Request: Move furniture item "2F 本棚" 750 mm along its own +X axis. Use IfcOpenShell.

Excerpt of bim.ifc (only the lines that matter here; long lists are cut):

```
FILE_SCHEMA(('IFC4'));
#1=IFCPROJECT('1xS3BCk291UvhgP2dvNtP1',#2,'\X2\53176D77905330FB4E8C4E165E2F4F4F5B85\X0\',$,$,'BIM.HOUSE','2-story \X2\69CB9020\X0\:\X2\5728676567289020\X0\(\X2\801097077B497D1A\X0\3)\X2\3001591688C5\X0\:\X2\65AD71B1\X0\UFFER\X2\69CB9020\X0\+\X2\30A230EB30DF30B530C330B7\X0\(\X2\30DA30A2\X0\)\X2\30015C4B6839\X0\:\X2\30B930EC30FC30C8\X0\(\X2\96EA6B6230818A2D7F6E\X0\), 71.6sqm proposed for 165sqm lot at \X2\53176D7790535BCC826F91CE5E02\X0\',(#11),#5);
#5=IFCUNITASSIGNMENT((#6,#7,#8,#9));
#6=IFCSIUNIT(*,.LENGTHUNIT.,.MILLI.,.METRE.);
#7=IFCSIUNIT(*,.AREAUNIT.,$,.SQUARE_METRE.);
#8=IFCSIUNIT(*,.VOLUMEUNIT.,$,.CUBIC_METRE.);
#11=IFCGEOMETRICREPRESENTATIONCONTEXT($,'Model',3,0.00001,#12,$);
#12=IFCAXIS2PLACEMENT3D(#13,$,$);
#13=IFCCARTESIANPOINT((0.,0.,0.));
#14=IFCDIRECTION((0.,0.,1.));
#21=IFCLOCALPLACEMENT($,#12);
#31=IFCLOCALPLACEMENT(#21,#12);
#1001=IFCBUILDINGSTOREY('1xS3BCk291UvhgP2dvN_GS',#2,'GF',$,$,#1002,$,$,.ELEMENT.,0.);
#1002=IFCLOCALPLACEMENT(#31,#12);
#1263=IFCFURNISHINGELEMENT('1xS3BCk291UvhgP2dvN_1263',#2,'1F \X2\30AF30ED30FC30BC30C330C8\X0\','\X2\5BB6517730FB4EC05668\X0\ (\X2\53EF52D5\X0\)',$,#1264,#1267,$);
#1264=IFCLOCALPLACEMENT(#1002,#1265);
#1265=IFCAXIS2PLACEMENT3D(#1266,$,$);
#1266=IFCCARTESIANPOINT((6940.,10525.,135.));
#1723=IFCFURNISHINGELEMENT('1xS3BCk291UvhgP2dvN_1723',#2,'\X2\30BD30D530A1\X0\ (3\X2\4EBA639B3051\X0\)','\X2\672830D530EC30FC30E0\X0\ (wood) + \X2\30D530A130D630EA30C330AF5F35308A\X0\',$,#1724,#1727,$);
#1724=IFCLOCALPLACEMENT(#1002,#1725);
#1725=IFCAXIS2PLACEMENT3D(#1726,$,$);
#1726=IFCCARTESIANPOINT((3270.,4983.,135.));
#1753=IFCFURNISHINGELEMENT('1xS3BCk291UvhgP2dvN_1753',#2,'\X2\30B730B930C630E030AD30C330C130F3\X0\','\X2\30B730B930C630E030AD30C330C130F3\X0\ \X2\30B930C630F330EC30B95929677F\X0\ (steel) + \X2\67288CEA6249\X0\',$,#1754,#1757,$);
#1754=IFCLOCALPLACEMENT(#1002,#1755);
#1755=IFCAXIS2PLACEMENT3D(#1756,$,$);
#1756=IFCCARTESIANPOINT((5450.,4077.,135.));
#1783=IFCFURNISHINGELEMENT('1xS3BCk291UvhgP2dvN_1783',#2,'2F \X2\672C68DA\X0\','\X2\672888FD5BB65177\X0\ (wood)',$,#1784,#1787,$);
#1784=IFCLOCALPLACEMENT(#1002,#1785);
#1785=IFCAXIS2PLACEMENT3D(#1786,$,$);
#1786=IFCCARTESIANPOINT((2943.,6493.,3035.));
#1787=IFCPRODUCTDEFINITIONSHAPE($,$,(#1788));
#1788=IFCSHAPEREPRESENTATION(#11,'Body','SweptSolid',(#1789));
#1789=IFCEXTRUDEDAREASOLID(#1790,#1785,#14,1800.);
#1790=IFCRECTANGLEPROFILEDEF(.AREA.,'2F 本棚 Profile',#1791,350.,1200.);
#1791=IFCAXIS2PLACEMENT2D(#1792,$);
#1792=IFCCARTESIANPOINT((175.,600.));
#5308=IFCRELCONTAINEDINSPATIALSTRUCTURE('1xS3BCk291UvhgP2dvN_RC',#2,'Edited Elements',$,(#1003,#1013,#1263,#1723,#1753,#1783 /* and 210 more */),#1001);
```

```python
import ifcopenshell
import ifcopenshell.api.geometry
import ifcopenshell.util.placement

model = ifcopenshell.open("bim.ifc")

item = model.by_guid("1xS3BCk291UvhgP2dvN_1783")
matrix = ifcopenshell.util.placement.get_local_placement(item.ObjectPlacement)
matrix[:3, 3] += matrix[:3, 0] * 750.0
ifcopenshell.api.geometry.edit_object_placement(model, product=item, matrix=matrix, is_si=False)

print(ifcopenshell.util.placement.get_local_placement(item.ObjectPlacement).round(3) + 0.0)

model.write("bim-out.ifc")
```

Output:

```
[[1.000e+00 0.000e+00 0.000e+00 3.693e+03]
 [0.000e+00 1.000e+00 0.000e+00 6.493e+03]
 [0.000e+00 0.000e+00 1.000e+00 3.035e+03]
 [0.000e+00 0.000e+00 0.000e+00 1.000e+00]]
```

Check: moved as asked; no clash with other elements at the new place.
